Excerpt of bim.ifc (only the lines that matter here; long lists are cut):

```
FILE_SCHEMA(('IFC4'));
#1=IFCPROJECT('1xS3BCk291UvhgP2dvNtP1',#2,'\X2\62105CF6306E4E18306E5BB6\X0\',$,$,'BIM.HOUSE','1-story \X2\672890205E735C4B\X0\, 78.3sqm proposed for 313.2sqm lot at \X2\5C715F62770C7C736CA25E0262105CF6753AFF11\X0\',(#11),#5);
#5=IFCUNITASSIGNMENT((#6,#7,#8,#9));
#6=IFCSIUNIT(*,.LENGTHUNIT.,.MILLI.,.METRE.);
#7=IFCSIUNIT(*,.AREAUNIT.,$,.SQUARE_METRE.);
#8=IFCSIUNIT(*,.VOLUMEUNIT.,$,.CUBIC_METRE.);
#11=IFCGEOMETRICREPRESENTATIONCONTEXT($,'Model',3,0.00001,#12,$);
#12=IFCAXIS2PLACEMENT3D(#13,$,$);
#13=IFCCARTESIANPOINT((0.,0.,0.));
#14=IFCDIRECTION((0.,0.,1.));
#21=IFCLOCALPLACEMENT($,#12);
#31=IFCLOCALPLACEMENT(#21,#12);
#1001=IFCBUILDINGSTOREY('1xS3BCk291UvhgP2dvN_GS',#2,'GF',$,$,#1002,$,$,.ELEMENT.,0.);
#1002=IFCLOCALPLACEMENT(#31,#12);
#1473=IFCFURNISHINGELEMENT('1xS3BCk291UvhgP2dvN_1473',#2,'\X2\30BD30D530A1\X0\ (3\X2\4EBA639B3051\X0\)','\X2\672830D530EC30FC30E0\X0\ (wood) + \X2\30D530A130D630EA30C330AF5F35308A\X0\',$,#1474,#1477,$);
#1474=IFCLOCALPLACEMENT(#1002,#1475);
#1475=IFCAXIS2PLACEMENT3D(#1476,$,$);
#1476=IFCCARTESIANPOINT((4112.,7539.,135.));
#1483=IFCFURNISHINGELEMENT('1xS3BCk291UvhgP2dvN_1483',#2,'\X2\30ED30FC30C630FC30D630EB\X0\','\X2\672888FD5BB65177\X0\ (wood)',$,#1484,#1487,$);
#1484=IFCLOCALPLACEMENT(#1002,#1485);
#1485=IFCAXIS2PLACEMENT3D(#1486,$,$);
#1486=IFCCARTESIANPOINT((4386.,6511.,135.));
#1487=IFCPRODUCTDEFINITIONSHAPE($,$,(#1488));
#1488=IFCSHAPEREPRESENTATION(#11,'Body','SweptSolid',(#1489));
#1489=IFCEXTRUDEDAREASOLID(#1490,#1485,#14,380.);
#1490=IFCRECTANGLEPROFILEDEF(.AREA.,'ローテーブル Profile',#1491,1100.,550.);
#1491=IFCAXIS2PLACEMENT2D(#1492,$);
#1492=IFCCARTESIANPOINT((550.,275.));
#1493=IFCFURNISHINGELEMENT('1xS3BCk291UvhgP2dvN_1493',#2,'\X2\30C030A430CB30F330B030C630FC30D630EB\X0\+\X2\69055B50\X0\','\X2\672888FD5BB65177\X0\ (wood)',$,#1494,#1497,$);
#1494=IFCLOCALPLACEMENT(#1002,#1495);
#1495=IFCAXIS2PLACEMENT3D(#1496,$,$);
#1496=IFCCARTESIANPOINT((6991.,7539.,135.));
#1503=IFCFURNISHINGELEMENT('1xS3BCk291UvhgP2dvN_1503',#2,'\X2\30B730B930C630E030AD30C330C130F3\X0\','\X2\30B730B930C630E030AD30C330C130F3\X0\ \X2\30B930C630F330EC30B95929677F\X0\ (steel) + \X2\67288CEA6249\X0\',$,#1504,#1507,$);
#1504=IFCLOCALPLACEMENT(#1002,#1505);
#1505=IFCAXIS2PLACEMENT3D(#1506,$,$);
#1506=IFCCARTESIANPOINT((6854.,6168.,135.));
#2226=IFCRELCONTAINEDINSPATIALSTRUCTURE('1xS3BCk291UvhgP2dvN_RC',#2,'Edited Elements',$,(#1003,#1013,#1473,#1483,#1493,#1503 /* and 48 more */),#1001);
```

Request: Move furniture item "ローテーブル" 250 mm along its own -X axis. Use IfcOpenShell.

```python
import ifcopenshell
import ifcopenshell.api.geometry
import ifcopenshell.util.placement
import ifcopenshell.util.unit

model = ifcopenshell.open("bim.ifc")
unit_scale = ifcopenshell.util.unit.calculate_unit_scale(model)

item = model.by_guid("1xS3BCk291UvhgP2dvN_1483")
matrix = ifcopenshell.util.placement.get_local_placement(item.ObjectPlacement)
matrix[:3, 3] -= matrix[:3, 0] * 0.25 / unit_scale
ifcopenshell.api.geometry.edit_object_placement(model, product=item, matrix=matrix, is_si=False)

print(ifcopenshell.util.placement.get_local_placement(item.ObjectPlacement).round(3) + 0.0)

model.write("bim_updated.ifc")
```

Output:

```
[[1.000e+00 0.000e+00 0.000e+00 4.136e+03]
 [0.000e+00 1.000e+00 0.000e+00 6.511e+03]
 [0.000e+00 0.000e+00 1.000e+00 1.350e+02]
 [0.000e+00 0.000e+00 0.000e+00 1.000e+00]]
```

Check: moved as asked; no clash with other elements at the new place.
